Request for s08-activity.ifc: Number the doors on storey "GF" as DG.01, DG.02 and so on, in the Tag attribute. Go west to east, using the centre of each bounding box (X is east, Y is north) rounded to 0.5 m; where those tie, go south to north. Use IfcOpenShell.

First a look at what the model holds.

```python
import ifcopenshell
import ifcopenshell.util.element
import ifcopenshell.util.placement

model = ifcopenshell.open("s08-activity.ifc")
print(model.schema)
storey = next(s for s in model.by_type("IfcBuildingStorey") if s.Name == "GF")
doors = [e for e in ifcopenshell.util.element.get_decomposition(storey) if e.is_a("IfcDoor")]
for e in sorted(doors, key=lambda e: e.id()):
    origin = ifcopenshell.util.placement.get_local_placement(e.ObjectPlacement)[:3, 3]
    print(e.id(), e.Tag, e.Name, origin.round(2) + 0.0, sep=" | ")
```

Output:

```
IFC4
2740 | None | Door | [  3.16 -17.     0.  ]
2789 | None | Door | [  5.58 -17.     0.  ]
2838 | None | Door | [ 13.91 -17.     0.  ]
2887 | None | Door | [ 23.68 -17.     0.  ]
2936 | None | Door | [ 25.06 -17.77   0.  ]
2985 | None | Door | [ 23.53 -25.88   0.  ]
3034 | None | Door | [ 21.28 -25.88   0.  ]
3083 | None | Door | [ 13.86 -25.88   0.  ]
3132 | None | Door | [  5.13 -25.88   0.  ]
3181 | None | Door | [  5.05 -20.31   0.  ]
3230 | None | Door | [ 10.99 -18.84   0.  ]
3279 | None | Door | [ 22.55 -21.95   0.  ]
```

```python
import ifcopenshell
import ifcopenshell.geom
import ifcopenshell.util.element
import ifcopenshell.util.shape

model = ifcopenshell.open("s08-activity.ifc")
settings = ifcopenshell.geom.settings()
settings.set("use-world-coords", True)


def centre(element):
    shape = ifcopenshell.geom.create_shape(settings, element)
    return ifcopenshell.util.shape.get_bbox_centroid(shape.geometry)


storey = next(s for s in model.by_type("IfcBuildingStorey") if s.Name == "GF")
doors = [e for e in ifcopenshell.util.element.get_decomposition(storey) if e.is_a("IfcDoor")]

# Insertion points can sit at a corner or the storey origin, so sort by the geometry (in metres).
centres = {e: centre(e) for e in doors}
doors.sort(key=lambda e: (round(centres[e][0] / 0.5), centres[e][1]))

for i, e in enumerate(doors, start=1):
    number = f"DG.{i:02d}"
    e.Tag = number
    print(e.id(), number)

model.write("s08-activity_v2.ifc")
```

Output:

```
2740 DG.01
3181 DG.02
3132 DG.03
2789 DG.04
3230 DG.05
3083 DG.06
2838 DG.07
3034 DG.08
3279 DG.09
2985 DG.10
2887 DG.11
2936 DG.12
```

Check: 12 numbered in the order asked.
